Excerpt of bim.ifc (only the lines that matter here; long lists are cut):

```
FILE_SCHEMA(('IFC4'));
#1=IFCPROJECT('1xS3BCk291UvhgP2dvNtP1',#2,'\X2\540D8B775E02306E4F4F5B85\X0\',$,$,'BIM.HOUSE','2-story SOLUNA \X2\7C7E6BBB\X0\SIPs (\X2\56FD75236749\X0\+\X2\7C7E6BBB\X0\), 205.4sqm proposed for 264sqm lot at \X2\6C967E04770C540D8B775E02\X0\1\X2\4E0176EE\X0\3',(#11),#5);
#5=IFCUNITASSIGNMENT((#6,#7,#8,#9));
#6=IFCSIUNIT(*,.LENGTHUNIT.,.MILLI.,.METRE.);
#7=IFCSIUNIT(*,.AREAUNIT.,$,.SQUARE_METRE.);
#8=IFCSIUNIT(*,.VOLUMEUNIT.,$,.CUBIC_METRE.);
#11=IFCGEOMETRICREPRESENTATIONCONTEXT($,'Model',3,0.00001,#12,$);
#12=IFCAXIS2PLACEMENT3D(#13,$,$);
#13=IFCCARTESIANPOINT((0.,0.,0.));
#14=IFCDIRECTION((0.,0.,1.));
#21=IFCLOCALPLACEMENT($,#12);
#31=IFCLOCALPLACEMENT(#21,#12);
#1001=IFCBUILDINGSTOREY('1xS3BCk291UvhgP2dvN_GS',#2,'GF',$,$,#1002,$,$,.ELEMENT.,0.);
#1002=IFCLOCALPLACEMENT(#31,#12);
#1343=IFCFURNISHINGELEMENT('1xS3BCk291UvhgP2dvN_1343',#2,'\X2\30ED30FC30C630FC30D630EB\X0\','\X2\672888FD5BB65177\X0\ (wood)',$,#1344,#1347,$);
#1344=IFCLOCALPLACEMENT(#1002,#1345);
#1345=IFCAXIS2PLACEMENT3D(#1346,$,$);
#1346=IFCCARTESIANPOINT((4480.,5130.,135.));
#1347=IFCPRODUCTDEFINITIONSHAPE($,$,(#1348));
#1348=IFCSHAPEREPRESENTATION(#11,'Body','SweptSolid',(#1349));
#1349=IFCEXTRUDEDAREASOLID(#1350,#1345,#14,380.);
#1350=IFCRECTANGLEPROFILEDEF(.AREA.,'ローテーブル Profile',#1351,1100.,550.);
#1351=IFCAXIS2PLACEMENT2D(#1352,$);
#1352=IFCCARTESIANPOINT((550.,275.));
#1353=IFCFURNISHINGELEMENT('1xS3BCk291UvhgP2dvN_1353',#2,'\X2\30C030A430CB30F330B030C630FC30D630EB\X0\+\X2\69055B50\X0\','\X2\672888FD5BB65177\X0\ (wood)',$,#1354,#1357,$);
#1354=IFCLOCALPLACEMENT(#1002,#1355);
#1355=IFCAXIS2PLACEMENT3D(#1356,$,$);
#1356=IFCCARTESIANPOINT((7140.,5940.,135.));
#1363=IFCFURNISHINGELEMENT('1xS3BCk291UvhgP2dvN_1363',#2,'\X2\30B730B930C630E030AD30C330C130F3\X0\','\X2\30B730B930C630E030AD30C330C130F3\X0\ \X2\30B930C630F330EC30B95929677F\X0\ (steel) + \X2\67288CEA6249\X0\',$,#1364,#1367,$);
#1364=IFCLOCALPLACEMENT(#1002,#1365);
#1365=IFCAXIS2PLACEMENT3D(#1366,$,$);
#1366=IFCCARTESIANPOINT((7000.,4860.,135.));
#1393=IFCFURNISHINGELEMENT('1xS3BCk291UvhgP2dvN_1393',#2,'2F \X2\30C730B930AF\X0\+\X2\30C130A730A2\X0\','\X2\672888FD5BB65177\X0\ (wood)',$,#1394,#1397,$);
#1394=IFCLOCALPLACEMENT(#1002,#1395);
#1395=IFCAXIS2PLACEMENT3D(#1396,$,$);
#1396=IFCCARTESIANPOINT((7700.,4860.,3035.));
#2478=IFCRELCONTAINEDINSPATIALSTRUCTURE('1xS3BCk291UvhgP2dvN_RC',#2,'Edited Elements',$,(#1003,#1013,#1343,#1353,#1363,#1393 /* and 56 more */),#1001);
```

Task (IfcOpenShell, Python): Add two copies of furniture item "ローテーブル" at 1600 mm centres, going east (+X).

```python
import numpy as np
import ifcopenshell
import ifcopenshell.api.geometry
import ifcopenshell.api.root
import ifcopenshell.util.element
import ifcopenshell.util.placement
import ifcopenshell.util.unit

model = ifcopenshell.open("bim.ifc")
unit_scale = ifcopenshell.util.unit.calculate_unit_scale(model)


def reuse_history(source, copy):
    """copy_class also copies each property set's owner history, people and application; keep the originals."""
    for rel in copy.IsDefinedBy:
        if rel.is_a("IfcRelDefinesByProperties") and (history := rel.RelatingPropertyDefinition.OwnerHistory):
            rel.RelatingPropertyDefinition.OwnerHistory = source.OwnerHistory
            ifcopenshell.util.element.remove_deep2(model, history)


source = model.by_id(1343)
base = ifcopenshell.util.placement.get_local_placement(source.ObjectPlacement)
step = np.array([1.0, 0.0, 0.0]) * 1.6 / unit_scale

for i in range(1, 3):
    copy = ifcopenshell.api.root.copy_class(model, product=source)
    copy.Representation = ifcopenshell.util.element.copy_deep(
        model, source.Representation, exclude=["IfcGeometricRepresentationContext", "IfcRepresentationMap"]
    )
    reuse_history(source, copy)
    matrix = base.copy()
    matrix[:3, 3] += i * step
    print("added at", matrix[:3, 3].round(3) + 0.0)
    ifcopenshell.api.geometry.edit_object_placement(model, product=copy, matrix=matrix, is_si=False)

model.write("bim_updated.ifc")
```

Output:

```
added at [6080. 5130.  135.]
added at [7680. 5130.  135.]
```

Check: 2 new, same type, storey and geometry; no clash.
